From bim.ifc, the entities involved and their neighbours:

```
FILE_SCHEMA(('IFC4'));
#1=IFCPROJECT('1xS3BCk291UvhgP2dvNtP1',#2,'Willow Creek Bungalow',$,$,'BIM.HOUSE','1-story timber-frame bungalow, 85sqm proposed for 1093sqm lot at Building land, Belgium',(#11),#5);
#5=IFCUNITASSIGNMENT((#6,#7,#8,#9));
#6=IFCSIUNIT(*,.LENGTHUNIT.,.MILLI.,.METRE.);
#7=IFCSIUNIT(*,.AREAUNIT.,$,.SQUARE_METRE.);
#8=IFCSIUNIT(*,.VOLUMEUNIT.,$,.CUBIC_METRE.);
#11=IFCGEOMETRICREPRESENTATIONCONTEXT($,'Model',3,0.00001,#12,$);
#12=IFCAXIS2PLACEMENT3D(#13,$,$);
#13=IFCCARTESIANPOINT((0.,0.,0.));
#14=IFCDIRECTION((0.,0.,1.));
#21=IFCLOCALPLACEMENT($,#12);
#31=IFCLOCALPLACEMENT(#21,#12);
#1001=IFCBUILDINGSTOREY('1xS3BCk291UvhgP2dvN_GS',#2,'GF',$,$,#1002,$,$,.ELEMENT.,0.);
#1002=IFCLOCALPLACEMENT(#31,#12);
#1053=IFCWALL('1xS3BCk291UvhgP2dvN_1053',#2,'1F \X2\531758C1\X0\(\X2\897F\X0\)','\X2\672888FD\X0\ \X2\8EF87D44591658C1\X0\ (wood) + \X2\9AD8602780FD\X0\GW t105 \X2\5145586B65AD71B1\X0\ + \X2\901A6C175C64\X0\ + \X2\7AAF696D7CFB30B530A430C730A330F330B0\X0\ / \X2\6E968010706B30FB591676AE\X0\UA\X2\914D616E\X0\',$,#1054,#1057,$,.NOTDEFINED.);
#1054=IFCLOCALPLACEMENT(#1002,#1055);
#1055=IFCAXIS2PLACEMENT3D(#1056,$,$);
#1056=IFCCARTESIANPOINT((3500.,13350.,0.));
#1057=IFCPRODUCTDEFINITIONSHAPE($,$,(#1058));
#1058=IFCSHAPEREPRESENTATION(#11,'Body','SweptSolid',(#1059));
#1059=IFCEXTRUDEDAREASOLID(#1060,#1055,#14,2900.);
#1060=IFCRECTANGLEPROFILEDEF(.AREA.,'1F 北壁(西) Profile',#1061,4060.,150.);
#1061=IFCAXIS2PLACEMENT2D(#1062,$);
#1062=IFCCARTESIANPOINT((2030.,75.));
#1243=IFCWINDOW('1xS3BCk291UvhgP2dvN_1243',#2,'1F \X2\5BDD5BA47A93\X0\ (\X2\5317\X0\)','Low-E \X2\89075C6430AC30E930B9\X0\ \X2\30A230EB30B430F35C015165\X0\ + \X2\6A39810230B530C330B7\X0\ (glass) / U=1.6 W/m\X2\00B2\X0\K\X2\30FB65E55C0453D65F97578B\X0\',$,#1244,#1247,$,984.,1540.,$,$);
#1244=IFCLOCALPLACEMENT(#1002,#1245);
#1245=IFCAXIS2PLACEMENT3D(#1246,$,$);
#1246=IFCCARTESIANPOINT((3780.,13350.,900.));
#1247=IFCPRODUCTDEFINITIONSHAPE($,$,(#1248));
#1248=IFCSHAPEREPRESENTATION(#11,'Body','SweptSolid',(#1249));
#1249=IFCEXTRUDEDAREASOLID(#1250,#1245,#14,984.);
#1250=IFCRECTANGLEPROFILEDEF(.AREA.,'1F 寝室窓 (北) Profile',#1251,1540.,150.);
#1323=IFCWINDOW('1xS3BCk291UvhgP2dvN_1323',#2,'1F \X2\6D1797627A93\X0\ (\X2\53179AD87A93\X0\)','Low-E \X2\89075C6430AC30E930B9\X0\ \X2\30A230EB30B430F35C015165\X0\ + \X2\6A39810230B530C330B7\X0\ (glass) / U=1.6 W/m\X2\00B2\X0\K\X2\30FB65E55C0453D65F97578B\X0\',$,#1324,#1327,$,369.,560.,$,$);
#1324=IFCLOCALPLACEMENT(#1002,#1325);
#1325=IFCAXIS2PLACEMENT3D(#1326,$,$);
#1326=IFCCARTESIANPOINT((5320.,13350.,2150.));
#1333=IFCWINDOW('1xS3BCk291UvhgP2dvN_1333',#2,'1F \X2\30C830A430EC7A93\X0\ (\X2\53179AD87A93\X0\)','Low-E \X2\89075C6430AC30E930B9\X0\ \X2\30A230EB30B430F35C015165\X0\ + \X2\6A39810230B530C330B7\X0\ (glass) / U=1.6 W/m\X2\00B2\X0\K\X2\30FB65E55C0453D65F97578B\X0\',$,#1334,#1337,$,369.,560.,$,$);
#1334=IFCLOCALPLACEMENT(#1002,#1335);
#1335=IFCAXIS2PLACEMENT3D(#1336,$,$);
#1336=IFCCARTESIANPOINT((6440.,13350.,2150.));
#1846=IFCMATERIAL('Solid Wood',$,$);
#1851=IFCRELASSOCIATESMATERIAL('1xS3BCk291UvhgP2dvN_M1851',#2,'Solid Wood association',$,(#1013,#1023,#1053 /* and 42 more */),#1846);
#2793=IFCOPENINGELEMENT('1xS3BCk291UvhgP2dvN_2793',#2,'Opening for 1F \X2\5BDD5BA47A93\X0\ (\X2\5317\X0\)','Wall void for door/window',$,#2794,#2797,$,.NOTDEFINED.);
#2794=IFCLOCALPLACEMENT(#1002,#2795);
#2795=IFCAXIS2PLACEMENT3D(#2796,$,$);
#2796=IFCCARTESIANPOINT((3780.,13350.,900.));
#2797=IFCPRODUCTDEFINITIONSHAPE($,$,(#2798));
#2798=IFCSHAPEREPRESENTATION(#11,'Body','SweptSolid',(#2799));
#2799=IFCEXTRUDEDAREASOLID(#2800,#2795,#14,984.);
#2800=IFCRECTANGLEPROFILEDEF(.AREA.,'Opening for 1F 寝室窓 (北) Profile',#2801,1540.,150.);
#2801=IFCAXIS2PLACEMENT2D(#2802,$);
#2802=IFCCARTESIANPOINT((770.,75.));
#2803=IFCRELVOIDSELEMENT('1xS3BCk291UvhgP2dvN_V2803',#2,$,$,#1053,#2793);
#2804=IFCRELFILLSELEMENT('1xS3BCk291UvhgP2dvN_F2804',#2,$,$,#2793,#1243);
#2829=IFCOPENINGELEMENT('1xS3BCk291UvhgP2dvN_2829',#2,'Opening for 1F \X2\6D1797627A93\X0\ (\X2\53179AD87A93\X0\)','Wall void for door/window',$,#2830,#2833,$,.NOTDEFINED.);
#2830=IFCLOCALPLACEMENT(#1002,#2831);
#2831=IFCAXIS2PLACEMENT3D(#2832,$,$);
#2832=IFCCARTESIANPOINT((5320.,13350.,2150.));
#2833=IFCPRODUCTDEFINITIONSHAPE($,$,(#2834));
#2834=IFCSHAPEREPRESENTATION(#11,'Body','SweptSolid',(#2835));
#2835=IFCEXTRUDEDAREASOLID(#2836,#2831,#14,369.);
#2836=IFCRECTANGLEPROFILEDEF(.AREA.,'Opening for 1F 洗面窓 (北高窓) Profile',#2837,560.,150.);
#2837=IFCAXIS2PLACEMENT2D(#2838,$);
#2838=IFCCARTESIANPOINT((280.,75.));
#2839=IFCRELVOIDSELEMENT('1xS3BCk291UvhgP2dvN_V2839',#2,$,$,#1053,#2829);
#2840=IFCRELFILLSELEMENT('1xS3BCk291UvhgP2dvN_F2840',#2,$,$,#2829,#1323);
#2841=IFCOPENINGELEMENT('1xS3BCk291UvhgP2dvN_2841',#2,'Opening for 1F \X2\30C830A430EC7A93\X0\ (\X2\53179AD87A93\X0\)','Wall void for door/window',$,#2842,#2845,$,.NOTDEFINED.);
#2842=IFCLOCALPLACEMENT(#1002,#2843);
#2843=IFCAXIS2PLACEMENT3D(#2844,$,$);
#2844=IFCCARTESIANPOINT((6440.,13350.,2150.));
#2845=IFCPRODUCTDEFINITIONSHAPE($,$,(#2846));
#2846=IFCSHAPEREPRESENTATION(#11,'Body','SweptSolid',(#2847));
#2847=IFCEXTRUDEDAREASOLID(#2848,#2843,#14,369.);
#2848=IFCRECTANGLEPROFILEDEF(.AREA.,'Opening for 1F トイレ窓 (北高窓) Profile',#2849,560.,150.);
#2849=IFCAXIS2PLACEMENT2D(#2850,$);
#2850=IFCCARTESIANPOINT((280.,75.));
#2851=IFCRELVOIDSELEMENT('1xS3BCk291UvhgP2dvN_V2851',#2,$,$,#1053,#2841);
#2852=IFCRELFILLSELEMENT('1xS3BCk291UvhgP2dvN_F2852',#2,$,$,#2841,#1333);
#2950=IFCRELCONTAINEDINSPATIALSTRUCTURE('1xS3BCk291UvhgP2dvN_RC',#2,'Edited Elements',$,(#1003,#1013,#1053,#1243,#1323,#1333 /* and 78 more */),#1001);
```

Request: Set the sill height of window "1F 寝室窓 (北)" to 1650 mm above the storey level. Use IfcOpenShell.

```python
import numpy as np
import ifcopenshell
import ifcopenshell.api.geometry
import ifcopenshell.geom
import ifcopenshell.util.element
import ifcopenshell.util.placement
import ifcopenshell.util.shape
import ifcopenshell.util.unit

model = ifcopenshell.open("bim.ifc")
unit_scale = ifcopenshell.util.unit.calculate_unit_scale(model)

window = model.by_guid("1xS3BCk291UvhgP2dvN_1243")
opening = window.FillsVoids[0].RelatingOpeningElement
storey = ifcopenshell.util.element.get_container(window, ifc_class="IfcBuildingStorey")
level = ifcopenshell.util.placement.get_local_placement(storey.ObjectPlacement)[2, 3]

# The opening's origin need not be at the sill, so measure its lowest point.
shape = ifcopenshell.geom.create_shape(ifcopenshell.geom.settings(), opening)
bottom = ifcopenshell.util.shape.get_shape_bottom_elevation(shape, shape.geometry) / unit_scale
dz = level + 1.65 / unit_scale - bottom

shift = np.array([0.0, 0.0, dz])
# The window is not placed relative to its opening, so move both.
for product in (opening, window):
    matrix = ifcopenshell.util.placement.get_local_placement(product.ObjectPlacement)
    matrix[:3, 3] += shift
    ifcopenshell.api.geometry.edit_object_placement(model, product=product, matrix=matrix, is_si=False)

print(f"moved by {dz * unit_scale:+.3f} m")

model.write("bim_updated.ifc")
```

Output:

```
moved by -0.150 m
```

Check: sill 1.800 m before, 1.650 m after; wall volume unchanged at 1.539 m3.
